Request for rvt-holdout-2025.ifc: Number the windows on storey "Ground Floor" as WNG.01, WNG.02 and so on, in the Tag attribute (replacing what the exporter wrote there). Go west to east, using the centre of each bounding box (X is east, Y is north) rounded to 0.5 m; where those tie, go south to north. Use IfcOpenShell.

First a look at what the model holds.

```python
import ifcopenshell
import ifcopenshell.util.element
import ifcopenshell.util.placement

model = ifcopenshell.open("rvt-holdout-2025.ifc")
print(model.schema)
storey = next(s for s in model.by_type("IfcBuildingStorey") if s.Name == "Ground Floor")
windows = [e for e in ifcopenshell.util.element.get_decomposition(storey) if e.is_a("IfcWindow")]
for e in sorted(windows, key=lambda e: e.id()):
    origin = ifcopenshell.util.placement.get_local_placement(e.ObjectPlacement)[:3, 3]
    print(e.id(), e.Tag, e.Name, origin.round(2) + 0.0, sep=" | ")
```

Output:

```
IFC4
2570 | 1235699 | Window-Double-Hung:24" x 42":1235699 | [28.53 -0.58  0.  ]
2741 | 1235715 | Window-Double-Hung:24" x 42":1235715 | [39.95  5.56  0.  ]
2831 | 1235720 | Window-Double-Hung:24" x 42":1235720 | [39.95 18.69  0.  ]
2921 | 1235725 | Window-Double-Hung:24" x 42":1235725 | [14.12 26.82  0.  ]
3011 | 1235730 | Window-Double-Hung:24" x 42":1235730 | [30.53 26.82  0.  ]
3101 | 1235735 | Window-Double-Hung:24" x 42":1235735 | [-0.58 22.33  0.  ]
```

```python
import ifcopenshell
import ifcopenshell.geom
import ifcopenshell.util.element
import ifcopenshell.util.shape

model = ifcopenshell.open("rvt-holdout-2025.ifc")
settings = ifcopenshell.geom.settings()
settings.set("use-world-coords", True)


def centre(element):
    shape = ifcopenshell.geom.create_shape(settings, element)
    return ifcopenshell.util.shape.get_bbox_centroid(shape.geometry)


storey = next(s for s in model.by_type("IfcBuildingStorey") if s.Name == "Ground Floor")
windows = [e for e in ifcopenshell.util.element.get_decomposition(storey) if e.is_a("IfcWindow")]

# Insertion points can sit at a corner or the storey origin, so sort by the geometry (in metres).
centres = {e: centre(e) for e in windows}
windows.sort(key=lambda e: (round(centres[e][0] / 0.5), centres[e][1]))

for i, e in enumerate(windows, start=1):
    number = f"WNG.{i:02d}"
    e.Tag = number
    print(e.id(), number)

model.write("rvt-holdout-2025_v2.ifc")
```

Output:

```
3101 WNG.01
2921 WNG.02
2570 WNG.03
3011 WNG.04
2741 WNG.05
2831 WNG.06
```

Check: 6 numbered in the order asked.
